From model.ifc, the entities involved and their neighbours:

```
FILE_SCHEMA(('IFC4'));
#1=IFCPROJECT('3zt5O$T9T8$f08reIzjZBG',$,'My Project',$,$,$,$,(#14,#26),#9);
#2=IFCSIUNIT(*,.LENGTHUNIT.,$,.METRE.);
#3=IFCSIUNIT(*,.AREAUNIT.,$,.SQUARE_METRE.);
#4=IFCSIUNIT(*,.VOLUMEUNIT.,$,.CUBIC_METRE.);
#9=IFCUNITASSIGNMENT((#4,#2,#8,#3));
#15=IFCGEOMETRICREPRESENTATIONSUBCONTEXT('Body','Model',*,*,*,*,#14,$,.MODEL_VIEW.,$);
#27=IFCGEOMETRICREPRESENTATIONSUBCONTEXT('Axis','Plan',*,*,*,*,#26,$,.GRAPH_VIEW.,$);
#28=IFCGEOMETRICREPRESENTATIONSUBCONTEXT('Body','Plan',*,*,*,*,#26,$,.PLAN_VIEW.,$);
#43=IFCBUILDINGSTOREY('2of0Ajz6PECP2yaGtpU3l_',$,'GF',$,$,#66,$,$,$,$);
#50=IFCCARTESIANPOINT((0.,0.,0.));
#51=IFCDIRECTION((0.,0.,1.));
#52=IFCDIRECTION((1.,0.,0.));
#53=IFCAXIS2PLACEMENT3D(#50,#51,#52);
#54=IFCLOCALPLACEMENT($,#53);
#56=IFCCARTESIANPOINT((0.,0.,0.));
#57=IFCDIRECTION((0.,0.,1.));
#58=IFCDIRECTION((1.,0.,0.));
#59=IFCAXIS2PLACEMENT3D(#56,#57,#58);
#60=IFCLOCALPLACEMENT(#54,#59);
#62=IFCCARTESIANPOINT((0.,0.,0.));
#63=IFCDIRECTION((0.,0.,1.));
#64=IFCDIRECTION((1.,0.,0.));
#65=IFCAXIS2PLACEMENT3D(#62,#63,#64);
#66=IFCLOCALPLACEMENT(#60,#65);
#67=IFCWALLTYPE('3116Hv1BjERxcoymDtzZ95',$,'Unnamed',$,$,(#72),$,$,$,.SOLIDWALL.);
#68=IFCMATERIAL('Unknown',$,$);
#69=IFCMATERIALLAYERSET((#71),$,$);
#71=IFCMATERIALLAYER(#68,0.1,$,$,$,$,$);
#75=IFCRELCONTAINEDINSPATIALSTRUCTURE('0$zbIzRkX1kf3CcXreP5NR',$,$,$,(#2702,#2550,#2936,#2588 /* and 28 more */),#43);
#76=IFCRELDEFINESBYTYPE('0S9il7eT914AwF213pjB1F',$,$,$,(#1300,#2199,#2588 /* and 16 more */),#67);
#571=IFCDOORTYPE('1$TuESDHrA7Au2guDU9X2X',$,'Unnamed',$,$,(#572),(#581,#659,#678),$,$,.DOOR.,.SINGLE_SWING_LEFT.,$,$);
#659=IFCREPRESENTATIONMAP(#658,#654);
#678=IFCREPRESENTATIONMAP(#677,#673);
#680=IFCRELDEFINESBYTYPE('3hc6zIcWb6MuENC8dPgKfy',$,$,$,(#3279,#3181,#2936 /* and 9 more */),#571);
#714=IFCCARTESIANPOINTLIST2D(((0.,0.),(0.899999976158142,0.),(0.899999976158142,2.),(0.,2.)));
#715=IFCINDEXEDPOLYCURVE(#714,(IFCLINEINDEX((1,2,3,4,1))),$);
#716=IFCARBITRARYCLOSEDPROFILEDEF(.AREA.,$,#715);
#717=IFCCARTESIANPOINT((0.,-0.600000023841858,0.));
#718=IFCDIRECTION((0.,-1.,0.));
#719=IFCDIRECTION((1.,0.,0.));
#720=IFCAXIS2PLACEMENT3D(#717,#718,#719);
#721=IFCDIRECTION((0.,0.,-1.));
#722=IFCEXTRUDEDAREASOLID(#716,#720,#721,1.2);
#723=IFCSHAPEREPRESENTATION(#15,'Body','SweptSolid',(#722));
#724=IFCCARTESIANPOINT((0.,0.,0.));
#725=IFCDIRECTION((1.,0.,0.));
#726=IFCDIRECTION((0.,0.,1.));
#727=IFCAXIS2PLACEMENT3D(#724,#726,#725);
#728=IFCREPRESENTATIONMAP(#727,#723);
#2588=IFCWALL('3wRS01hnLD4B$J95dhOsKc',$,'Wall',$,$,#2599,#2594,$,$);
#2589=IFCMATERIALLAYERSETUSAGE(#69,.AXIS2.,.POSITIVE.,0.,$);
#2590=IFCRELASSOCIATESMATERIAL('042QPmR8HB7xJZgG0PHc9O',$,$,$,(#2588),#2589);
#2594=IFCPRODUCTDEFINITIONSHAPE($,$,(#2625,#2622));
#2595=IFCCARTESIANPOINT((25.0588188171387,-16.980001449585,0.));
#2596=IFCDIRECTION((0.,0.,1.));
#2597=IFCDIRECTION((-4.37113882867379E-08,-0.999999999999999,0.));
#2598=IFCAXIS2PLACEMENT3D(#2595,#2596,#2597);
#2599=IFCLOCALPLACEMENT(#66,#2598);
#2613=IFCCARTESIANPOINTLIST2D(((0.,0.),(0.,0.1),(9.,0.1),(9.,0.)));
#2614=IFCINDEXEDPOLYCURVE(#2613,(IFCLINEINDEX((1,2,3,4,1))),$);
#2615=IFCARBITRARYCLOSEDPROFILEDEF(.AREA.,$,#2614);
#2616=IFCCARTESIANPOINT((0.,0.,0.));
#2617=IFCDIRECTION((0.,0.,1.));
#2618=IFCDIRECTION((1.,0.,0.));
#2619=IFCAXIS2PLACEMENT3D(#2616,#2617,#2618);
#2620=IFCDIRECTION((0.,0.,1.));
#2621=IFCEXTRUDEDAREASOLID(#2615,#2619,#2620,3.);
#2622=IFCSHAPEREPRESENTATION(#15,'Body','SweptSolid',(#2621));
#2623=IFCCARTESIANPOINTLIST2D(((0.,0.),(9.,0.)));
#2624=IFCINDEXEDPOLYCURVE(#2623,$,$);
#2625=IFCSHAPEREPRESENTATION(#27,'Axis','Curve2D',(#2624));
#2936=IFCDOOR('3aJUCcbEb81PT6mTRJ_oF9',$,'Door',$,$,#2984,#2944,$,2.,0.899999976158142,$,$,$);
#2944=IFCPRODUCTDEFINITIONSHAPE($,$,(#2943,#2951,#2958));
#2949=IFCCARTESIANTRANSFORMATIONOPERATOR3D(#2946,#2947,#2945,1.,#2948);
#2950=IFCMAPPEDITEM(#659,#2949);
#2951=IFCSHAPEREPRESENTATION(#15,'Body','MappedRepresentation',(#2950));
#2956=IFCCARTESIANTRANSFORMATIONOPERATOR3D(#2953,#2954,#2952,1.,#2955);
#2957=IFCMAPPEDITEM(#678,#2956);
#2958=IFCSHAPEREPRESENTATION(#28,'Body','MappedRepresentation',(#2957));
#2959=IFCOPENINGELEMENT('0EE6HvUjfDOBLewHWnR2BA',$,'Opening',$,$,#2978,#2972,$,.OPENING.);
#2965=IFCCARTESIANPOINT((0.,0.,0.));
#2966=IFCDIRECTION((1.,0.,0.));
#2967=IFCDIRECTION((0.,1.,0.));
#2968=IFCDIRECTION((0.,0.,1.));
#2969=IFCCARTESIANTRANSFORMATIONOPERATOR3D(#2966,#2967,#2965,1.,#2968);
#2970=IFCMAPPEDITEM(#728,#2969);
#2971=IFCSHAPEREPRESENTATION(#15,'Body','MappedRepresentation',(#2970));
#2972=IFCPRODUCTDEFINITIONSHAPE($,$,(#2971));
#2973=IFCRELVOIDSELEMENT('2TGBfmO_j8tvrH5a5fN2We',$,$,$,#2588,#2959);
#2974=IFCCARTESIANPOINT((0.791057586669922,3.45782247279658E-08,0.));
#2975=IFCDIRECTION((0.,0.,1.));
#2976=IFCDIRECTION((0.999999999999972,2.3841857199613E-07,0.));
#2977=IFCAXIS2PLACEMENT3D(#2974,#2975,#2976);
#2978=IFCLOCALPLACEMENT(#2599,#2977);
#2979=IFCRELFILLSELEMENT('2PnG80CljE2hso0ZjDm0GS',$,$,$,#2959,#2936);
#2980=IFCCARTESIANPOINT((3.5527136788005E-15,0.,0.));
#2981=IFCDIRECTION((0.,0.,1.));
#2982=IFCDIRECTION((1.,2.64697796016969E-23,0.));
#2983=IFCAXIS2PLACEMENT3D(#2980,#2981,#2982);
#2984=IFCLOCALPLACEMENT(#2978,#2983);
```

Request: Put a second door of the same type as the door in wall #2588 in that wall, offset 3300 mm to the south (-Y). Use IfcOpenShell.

```python
import ifcopenshell
import ifcopenshell.api.feature
import ifcopenshell.api.geometry
import ifcopenshell.api.root
import ifcopenshell.geom
import ifcopenshell.util.element
import ifcopenshell.util.placement
import ifcopenshell.util.shape

model = ifcopenshell.open("model.ifc")
settings = ifcopenshell.geom.settings()


def volume(element):
    """Net volume in cubic metres, openings subtracted."""
    shape = ifcopenshell.geom.create_shape(settings, element)
    return ifcopenshell.util.shape.get_volume(shape.geometry)


door = model.by_guid("3aJUCcbEb81PT6mTRJ_oF9")
opening = door.FillsVoids[0].RelatingOpeningElement
wall = opening.VoidsElements[0].RelatingBuildingElement
before = volume(wall)
shift = ifcopenshell.util.placement.get_local_placement(wall.ObjectPlacement)[:3, 0] * 3.3

# copy_class copies the void relationship, type, container and properties, but no geometry.
new_opening = ifcopenshell.api.root.copy_class(model, product=opening)
new_opening.Representation = ifcopenshell.util.element.copy_deep(
    model, opening.Representation, exclude=["IfcGeometricRepresentationContext", "IfcRepresentationMap"]
)
new_door = ifcopenshell.api.root.copy_class(model, product=door)
new_door.Representation = ifcopenshell.util.element.copy_deep(
    model, door.Representation, exclude=["IfcGeometricRepresentationContext", "IfcRepresentationMap"]
)
ifcopenshell.api.feature.add_filling(model, opening=new_opening, element=new_door)

for old, new in ((opening, new_opening), (door, new_door)):
    matrix = ifcopenshell.util.placement.get_local_placement(old.ObjectPlacement)
    matrix[:3, 3] += shift
    ifcopenshell.api.geometry.edit_object_placement(model, product=new, matrix=matrix, is_si=False)

after = volume(wall)

print(f"wall volume {before:.3f} -> {after:.3f} m3")

model.write("model_rev.ifc")
```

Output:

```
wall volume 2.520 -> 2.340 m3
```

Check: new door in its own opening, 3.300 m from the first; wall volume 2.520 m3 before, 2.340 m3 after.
